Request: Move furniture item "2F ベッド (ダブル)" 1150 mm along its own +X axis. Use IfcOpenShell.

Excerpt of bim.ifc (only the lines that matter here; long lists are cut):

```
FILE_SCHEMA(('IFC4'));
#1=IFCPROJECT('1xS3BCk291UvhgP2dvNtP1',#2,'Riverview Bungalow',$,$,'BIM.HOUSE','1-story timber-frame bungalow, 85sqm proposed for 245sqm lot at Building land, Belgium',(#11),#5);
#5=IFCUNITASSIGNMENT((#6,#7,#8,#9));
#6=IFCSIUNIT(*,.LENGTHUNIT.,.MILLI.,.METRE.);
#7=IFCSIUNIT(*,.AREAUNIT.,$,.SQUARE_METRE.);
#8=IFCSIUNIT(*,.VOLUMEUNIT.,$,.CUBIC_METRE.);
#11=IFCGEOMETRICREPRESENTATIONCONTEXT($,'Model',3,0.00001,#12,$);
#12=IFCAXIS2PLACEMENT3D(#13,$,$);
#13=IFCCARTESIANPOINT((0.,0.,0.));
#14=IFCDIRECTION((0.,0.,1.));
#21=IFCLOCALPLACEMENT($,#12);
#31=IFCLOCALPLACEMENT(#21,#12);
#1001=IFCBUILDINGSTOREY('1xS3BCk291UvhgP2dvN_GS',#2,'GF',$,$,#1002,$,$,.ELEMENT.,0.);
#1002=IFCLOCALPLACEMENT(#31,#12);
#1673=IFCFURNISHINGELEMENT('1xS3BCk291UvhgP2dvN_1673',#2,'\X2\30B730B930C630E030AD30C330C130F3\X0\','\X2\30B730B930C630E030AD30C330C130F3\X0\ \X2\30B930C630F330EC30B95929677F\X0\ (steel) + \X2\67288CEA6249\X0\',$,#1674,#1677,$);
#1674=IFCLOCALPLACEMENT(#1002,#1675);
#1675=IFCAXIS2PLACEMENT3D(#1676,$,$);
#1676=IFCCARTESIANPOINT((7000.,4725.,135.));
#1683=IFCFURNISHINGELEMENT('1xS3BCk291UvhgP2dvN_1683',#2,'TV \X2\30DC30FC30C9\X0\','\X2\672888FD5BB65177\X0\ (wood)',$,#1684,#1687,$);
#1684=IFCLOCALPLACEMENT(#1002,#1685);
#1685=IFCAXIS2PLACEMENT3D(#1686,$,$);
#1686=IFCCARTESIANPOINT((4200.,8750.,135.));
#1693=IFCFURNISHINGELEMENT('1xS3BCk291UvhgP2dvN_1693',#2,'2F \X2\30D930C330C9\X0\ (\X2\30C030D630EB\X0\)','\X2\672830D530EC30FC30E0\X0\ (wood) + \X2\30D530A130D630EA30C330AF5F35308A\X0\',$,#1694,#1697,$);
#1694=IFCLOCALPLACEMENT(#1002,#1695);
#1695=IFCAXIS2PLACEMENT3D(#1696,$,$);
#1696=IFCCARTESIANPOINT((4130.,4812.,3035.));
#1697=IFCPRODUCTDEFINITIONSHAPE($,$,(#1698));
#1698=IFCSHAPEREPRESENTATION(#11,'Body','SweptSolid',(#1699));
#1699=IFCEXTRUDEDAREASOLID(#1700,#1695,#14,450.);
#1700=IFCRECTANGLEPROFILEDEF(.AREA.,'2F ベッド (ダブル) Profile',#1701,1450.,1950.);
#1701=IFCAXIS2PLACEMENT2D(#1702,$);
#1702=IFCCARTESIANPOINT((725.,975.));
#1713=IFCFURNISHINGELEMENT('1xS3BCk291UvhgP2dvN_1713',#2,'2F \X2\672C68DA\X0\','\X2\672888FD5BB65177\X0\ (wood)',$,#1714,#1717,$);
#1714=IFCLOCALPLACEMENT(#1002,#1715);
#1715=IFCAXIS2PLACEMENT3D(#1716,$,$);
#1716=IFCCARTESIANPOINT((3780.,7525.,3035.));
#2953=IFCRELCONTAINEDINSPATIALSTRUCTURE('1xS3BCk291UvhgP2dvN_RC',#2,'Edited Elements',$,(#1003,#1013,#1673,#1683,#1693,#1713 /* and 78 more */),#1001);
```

```python
import ifcopenshell
import ifcopenshell.api.geometry
import ifcopenshell.util.placement
import ifcopenshell.util.unit

model = ifcopenshell.open("bim.ifc")
unit_scale = ifcopenshell.util.unit.calculate_unit_scale(model)

item = model.by_guid("1xS3BCk291UvhgP2dvN_1693")
matrix = ifcopenshell.util.placement.get_local_placement(item.ObjectPlacement)
matrix[:3, 3] += matrix[:3, 0] * 1.15 / unit_scale
ifcopenshell.api.geometry.edit_object_placement(model, product=item, matrix=matrix, is_si=False)

print(ifcopenshell.util.placement.get_local_placement(item.ObjectPlacement).round(3) + 0.0)

model.write("bim_rev.ifc")
```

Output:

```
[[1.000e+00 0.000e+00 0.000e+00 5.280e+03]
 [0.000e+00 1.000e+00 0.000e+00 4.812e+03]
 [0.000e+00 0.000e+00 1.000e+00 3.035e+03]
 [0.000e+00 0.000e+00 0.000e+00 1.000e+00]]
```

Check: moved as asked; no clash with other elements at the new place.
